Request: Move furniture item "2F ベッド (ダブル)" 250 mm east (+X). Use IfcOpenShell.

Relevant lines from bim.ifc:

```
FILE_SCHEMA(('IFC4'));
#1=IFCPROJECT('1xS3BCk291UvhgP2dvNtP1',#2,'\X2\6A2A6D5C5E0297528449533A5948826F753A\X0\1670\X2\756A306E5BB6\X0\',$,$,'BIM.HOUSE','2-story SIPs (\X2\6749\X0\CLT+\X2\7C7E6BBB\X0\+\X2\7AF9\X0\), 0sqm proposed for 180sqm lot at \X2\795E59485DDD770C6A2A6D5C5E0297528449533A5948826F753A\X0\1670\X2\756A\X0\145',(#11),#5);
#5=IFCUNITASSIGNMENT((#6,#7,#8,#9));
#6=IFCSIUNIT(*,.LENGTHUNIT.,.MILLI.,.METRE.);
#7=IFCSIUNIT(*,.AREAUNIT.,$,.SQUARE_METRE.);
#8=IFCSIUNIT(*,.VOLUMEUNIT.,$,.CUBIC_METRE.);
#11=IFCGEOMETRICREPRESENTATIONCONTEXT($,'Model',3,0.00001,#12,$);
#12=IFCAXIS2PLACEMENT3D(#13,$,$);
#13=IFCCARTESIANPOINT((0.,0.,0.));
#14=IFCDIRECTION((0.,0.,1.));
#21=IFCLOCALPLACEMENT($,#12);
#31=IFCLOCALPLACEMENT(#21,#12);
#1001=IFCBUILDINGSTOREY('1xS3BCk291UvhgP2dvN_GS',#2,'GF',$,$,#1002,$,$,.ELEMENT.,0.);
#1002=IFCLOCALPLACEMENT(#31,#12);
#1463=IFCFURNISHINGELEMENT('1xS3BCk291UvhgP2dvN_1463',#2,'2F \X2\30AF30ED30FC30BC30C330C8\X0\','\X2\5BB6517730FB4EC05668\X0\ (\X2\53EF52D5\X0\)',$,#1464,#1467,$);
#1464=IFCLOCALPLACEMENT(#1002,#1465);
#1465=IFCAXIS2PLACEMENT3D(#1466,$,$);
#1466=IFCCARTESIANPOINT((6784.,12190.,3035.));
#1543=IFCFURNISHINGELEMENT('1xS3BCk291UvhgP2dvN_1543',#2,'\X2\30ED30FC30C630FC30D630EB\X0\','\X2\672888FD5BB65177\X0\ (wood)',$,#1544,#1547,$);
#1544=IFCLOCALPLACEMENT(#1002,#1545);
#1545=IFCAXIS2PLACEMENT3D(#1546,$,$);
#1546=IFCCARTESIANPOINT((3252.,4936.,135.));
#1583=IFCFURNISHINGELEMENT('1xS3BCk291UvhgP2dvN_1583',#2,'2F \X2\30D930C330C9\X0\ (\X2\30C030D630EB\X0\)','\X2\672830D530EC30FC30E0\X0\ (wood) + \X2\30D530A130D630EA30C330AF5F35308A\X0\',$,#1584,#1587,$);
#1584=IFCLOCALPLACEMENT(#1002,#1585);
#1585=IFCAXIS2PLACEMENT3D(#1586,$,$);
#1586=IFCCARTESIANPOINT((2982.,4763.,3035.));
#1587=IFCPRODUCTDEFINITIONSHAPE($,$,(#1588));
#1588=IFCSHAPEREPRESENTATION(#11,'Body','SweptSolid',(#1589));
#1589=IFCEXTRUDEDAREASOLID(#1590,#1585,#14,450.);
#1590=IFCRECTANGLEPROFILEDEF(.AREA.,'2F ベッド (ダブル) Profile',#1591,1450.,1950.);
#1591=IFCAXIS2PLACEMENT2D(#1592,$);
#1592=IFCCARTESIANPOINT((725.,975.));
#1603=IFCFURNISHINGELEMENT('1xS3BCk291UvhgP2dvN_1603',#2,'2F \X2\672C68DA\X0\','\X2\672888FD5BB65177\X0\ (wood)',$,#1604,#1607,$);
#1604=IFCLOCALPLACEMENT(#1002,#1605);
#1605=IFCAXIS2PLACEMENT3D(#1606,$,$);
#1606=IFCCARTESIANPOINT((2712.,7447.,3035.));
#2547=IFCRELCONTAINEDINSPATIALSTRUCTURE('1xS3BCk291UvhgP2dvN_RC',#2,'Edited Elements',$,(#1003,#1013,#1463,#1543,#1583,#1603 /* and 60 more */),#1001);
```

```python
import ifcopenshell
import ifcopenshell.api.geometry
import ifcopenshell.util.placement

model = ifcopenshell.open("bim.ifc")

item = model.by_guid("1xS3BCk291UvhgP2dvN_1583")
matrix = ifcopenshell.util.placement.get_local_placement(item.ObjectPlacement)
matrix[0, 3] += 250.0
ifcopenshell.api.geometry.edit_object_placement(model, product=item, matrix=matrix, is_si=False)

print(ifcopenshell.util.placement.get_local_placement(item.ObjectPlacement).round(3) + 0.0)

model.write("bim_rev.ifc")
```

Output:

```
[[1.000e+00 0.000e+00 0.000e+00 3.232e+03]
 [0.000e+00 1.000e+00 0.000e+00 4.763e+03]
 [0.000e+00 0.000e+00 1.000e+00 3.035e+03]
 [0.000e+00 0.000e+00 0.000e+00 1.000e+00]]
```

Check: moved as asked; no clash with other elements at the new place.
